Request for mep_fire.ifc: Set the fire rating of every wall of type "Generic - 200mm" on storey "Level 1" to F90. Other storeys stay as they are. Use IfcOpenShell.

First a look at what the model holds.

```python
import ifcopenshell
import ifcopenshell.util.element

model = ifcopenshell.open("mep_fire.ifc")
print(model.schema)
storey = next(s for s in model.by_type("IfcBuildingStorey") if s.Name == "Level 1")
walls = [e for e in ifcopenshell.util.element.get_decomposition(storey) if e.is_a("IfcWall")]
seen = {}
for e in walls:
    element_type = ifcopenshell.util.element.get_type(e)
    key = (element_type.Name if element_type != e and element_type else None, ifcopenshell.util.element.get_pset(e, "Pset_WallCommon", "FireRating"))
    seen[key] = seen.get(key, 0) + 1
for (name, value), count in sorted(seen.items(), key=str):
    print(count, "x", name, "|", value)
```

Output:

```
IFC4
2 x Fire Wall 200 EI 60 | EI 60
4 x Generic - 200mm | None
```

```python
import ifcopenshell
import ifcopenshell.api.pset
import ifcopenshell.util.element

model = ifcopenshell.open("mep_fire.ifc")

storey = next(s for s in model.by_type("IfcBuildingStorey") if s.Name == "Level 1")
walls = [e for e in ifcopenshell.util.element.get_decomposition(storey) if e.is_a("IfcWall")]

count = 0
for e in walls:
    element_type = ifcopenshell.util.element.get_type(e)
    if element_type in (None, e) or element_type.Name != "Generic - 200mm":
        continue
    # add_pset returns the element's existing set when there is one.
    pset = ifcopenshell.api.pset.add_pset(model, product=e, name="Pset_WallCommon")
    ifcopenshell.api.pset.edit_pset(model, pset=pset, properties={"FireRating": "F90"})
    count += 1

print(count, "walls updated")

model.write("mep_fire_updated.ifc")
```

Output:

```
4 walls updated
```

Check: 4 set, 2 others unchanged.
